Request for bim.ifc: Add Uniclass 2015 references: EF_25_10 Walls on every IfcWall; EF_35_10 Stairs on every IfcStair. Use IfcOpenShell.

First a look at what the model holds.

```python
import ifcopenshell

model = ifcopenshell.open("bim.ifc")
print(model.schema)
print("classifications:", [c.Name for c in model.by_type("IfcClassification")])
for ifc_class in ("IfcDoor", "IfcRoof", "IfcStair", "IfcWall", "IfcWindow"):
    print(ifc_class, len(model.by_type(ifc_class)))
```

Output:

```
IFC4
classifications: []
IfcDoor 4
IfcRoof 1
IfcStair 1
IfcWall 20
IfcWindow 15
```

```python
import ifcopenshell
import ifcopenshell.api.classification

model = ifcopenshell.open("bim.ifc")

system = ifcopenshell.api.classification.add_classification(model, classification="Uniclass 2015")

codes = {
    "IfcWall": ("EF_25_10", "Walls"),
    "IfcStair": ("EF_35_10", "Stairs"),
}
for ifc_class, (code, name) in codes.items():
    products = model.by_type(ifc_class)
    ifcopenshell.api.classification.add_reference(
        model, products=products, classification=system, identification=code, name=name
    )
    print(code, len(products))

model.write("bim_v2.ifc")
```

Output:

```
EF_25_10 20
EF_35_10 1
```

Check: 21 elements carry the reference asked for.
